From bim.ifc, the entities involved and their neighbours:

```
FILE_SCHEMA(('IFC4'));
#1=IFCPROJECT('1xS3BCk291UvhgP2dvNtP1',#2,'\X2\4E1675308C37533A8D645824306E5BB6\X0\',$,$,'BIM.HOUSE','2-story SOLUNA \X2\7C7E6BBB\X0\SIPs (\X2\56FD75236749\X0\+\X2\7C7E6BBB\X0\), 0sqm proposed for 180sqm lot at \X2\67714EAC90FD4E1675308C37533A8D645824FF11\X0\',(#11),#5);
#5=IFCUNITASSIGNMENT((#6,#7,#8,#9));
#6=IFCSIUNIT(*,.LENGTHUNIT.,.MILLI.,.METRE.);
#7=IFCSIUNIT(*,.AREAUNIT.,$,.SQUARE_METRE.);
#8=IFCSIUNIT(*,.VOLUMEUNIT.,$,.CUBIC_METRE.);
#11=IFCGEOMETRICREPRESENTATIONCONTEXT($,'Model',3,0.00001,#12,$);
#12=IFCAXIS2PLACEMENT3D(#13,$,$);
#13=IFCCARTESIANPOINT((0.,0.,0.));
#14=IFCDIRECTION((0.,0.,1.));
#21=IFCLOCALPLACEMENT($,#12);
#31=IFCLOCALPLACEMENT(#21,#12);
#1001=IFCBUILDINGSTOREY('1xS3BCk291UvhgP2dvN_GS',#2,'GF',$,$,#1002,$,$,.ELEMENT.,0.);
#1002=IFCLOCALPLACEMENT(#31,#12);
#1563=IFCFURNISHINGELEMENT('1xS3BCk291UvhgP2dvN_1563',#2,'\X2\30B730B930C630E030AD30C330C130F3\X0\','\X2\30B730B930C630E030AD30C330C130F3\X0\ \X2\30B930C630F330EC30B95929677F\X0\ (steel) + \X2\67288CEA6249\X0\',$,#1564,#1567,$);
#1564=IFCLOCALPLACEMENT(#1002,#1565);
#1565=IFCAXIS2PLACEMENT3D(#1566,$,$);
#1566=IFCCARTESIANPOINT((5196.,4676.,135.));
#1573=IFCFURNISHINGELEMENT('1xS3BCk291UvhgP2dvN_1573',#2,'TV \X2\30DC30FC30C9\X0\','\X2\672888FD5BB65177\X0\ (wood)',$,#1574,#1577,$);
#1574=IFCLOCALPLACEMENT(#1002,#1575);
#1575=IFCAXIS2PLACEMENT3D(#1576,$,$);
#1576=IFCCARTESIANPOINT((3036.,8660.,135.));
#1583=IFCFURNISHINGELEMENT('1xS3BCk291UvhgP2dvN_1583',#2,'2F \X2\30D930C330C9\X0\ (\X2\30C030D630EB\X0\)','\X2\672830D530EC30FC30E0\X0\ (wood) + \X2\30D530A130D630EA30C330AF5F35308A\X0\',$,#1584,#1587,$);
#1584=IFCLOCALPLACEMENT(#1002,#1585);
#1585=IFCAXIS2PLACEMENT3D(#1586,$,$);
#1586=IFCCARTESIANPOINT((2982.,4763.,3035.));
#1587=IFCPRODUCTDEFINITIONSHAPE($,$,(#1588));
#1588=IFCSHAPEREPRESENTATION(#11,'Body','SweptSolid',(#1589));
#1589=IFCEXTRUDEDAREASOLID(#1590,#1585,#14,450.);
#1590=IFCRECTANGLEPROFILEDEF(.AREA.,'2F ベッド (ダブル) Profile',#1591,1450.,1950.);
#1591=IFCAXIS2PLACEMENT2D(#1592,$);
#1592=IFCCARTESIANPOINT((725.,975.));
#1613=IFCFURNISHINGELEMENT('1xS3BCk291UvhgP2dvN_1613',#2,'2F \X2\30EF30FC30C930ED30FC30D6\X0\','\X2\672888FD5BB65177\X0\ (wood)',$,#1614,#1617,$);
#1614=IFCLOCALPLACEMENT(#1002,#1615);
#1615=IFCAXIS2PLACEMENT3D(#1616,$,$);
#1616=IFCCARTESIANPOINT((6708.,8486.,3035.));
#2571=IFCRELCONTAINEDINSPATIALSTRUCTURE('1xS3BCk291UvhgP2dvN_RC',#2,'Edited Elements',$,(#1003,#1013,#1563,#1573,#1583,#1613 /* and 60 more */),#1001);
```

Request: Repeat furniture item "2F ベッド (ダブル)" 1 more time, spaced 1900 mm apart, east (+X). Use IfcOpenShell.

```python
import numpy as np
import ifcopenshell
import ifcopenshell.api.geometry
import ifcopenshell.api.root
import ifcopenshell.util.element
import ifcopenshell.util.placement

model = ifcopenshell.open("bim.ifc")


def reuse_history(source, copy):
    """copy_class also copies each property set's owner history, people and application; keep the originals."""
    for rel in copy.IsDefinedBy:
        if rel.is_a("IfcRelDefinesByProperties") and (history := rel.RelatingPropertyDefinition.OwnerHistory):
            rel.RelatingPropertyDefinition.OwnerHistory = source.OwnerHistory
            ifcopenshell.util.element.remove_deep2(model, history)


source = model.by_guid("1xS3BCk291UvhgP2dvN_1583")
base = ifcopenshell.util.placement.get_local_placement(source.ObjectPlacement)
step = np.array([1.0, 0.0, 0.0]) * 1900.0

for i in range(1, 2):
    copy = ifcopenshell.api.root.copy_class(model, product=source)
    copy.Representation = ifcopenshell.util.element.copy_deep(
        model, source.Representation, exclude=["IfcGeometricRepresentationContext", "IfcRepresentationMap"]
    )
    reuse_history(source, copy)
    matrix = base.copy()
    matrix[:3, 3] += i * step
    print("added at", matrix[:3, 3].round(3) + 0.0)
    ifcopenshell.api.geometry.edit_object_placement(model, product=copy, matrix=matrix, is_si=False)

model.write("bim-out.ifc")
```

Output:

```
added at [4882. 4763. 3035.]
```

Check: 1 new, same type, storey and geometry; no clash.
